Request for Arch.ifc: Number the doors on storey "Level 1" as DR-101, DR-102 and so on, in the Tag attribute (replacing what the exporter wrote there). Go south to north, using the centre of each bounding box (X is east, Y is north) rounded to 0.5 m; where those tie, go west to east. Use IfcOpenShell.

First a look at what the model holds.

```python
import ifcopenshell
import ifcopenshell.util.element
import ifcopenshell.util.placement

model = ifcopenshell.open("Arch.ifc")
print(model.schema)
storey = next(s for s in model.by_type("IfcBuildingStorey") if s.Name == "Level 1")
doors = [e for e in ifcopenshell.util.element.get_decomposition(storey) if e.is_a("IfcDoor")]
for e in sorted(doors, key=lambda e: e.id()):
    origin = ifcopenshell.util.placement.get_local_placement(e.ObjectPlacement)[:3, 3]
    print(e.id(), e.Tag, e.Name, origin.round(2) + 0.0, sep=" | ")
```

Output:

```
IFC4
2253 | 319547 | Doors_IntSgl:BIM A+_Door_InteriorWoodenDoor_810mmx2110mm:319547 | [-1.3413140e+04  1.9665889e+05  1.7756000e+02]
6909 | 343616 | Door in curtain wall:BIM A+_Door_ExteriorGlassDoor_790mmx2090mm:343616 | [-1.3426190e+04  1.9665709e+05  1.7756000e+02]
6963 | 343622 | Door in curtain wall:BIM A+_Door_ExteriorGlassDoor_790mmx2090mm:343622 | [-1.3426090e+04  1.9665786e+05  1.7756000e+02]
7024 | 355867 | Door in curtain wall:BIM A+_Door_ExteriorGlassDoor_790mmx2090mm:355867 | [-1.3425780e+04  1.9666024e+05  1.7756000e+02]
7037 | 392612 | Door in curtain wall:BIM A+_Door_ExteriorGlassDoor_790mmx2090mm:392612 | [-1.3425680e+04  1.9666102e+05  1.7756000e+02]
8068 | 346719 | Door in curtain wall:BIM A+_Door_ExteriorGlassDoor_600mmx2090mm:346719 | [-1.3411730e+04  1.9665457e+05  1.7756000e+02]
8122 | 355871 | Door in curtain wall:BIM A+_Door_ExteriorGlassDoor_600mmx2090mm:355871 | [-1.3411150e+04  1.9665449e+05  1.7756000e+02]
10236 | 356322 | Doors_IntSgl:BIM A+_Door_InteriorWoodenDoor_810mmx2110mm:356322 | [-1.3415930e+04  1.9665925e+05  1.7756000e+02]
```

```python
import ifcopenshell
import ifcopenshell.geom
import ifcopenshell.util.element
import ifcopenshell.util.shape

model = ifcopenshell.open("Arch.ifc")
settings = ifcopenshell.geom.settings()
settings.set("use-world-coords", True)


def centre(element):
    shape = ifcopenshell.geom.create_shape(settings, element)
    return ifcopenshell.util.shape.get_bbox_centroid(shape.geometry)


storey = next(s for s in model.by_type("IfcBuildingStorey") if s.Name == "Level 1")
doors = [e for e in ifcopenshell.util.element.get_decomposition(storey) if e.is_a("IfcDoor")]

# Insertion points can sit at a corner or the storey origin, so sort by the geometry (in metres).
centres = {e: centre(e) for e in doors}
doors.sort(key=lambda e: (round(centres[e][1] / 0.5), centres[e][0]))

for i, e in enumerate(doors, start=1):
    number = f"DR-1{i:02d}"
    e.Tag = number
    print(e.id(), number)

model.write("Arch_v2.ifc")
```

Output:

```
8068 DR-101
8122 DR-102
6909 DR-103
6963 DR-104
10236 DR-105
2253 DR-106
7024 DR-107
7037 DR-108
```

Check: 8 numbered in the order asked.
